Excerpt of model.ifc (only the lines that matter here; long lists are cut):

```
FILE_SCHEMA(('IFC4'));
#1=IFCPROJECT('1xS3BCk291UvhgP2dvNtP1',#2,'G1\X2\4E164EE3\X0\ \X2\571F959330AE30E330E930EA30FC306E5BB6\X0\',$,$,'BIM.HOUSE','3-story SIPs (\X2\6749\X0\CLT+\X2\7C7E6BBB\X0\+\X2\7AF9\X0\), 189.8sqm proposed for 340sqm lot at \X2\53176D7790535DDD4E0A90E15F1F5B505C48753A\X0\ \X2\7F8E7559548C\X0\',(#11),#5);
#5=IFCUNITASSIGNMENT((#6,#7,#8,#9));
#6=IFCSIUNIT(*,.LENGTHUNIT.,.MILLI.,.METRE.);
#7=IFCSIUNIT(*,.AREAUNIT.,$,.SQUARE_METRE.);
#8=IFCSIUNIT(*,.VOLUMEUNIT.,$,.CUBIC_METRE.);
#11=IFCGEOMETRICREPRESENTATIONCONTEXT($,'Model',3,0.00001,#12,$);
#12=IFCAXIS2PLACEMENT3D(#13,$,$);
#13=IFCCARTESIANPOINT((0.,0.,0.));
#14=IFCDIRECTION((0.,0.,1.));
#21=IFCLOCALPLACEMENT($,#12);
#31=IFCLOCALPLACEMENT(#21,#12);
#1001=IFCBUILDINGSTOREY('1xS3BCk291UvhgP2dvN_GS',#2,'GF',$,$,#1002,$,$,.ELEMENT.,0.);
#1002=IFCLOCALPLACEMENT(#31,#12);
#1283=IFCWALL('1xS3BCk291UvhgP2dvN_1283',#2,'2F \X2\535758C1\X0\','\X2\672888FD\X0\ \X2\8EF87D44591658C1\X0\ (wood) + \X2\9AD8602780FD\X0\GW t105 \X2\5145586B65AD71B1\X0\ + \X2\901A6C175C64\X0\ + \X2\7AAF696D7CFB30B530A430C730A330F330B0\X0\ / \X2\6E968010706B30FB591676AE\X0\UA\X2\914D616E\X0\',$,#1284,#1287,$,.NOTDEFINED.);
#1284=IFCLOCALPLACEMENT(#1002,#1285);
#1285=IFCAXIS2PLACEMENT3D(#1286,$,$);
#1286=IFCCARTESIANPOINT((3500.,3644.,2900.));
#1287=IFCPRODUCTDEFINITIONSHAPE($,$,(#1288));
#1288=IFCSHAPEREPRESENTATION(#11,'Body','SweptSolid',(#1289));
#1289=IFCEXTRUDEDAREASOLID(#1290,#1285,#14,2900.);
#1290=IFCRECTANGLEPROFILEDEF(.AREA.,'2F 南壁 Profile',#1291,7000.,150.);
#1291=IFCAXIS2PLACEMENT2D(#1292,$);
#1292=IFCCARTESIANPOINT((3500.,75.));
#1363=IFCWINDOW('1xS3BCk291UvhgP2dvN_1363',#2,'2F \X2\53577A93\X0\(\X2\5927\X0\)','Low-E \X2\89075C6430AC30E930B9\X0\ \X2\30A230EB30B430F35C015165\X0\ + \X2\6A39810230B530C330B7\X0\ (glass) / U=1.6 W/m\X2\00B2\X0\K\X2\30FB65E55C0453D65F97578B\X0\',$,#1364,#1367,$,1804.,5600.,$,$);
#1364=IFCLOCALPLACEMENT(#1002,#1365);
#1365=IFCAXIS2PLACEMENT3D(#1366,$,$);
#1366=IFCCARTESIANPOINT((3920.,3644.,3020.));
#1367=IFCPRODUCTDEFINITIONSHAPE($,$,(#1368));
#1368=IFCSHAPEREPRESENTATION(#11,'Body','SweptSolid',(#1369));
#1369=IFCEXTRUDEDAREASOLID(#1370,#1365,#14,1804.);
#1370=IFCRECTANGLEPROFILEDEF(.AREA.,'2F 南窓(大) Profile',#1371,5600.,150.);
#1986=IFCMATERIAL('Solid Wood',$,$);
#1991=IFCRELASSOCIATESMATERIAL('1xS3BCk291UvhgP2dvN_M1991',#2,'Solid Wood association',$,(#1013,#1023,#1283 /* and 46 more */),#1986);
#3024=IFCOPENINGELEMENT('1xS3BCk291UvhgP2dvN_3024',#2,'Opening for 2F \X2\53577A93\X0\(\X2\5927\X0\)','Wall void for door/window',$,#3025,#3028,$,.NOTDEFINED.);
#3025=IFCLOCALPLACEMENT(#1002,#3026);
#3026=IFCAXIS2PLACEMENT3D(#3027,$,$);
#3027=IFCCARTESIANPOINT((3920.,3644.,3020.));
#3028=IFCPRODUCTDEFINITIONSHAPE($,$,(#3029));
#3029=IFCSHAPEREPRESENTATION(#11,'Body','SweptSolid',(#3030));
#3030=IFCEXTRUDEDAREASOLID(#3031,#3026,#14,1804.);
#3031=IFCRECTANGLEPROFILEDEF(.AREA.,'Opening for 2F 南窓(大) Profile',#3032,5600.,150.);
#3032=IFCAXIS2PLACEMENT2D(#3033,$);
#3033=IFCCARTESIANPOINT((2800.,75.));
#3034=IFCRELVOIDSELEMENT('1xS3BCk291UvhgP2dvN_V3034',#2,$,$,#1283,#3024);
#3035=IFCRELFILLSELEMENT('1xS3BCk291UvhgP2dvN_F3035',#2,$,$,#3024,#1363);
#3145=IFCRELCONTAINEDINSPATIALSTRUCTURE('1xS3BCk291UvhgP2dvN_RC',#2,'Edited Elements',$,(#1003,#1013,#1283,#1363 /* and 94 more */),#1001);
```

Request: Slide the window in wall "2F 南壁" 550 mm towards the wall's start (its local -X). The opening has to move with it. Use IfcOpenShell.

```python
import ifcopenshell
import ifcopenshell.api.geometry
import ifcopenshell.util.placement
import ifcopenshell.util.unit

model = ifcopenshell.open("model.ifc")
unit_scale = ifcopenshell.util.unit.calculate_unit_scale(model)

window = model.by_id(1363)
opening = window.FillsVoids[0].RelatingOpeningElement
wall = opening.VoidsElements[0].RelatingBuildingElement

wall_matrix = ifcopenshell.util.placement.get_local_placement(wall.ObjectPlacement)
shift = wall_matrix[:3, 0] * -0.55 / unit_scale
before = ifcopenshell.util.placement.get_local_placement(window.ObjectPlacement)[:3, 3].copy()

# The window is not placed relative to its opening, so move both.
for product in (opening, window):
    matrix = ifcopenshell.util.placement.get_local_placement(product.ObjectPlacement)
    matrix[:3, 3] += shift
    ifcopenshell.api.geometry.edit_object_placement(model, product=product, matrix=matrix, is_si=False)

after = ifcopenshell.util.placement.get_local_placement(window.ObjectPlacement)[:3, 3]
print("window moved by", (after - before).round(3) + 0.0)

model.write("model-out.ifc")
```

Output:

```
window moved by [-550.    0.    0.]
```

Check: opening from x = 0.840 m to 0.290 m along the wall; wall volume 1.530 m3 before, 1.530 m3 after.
